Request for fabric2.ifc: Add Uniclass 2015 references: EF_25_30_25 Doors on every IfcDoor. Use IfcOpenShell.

First a look at what the model holds.

```python
import ifcopenshell

model = ifcopenshell.open("fabric2.ifc")
print(model.schema)
print("classifications:", [c.Name for c in model.by_type("IfcClassification")])
for ifc_class in ("IfcDoor", "IfcRoof", "IfcStair", "IfcWall", "IfcWindow"):
    print(ifc_class, len(model.by_type(ifc_class)))
```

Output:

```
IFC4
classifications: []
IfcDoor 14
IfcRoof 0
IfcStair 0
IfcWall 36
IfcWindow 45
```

```python
import ifcopenshell
import ifcopenshell.api.classification

model = ifcopenshell.open("fabric2.ifc")

system = ifcopenshell.api.classification.add_classification(model, classification="Uniclass 2015")

codes = {
    "IfcDoor": ("EF_25_30_25", "Doors"),
}
for ifc_class, (code, name) in codes.items():
    products = model.by_type(ifc_class)
    ifcopenshell.api.classification.add_reference(
        model, products=products, classification=system, identification=code, name=name
    )
    print(code, len(products))

model.write("fabric2_updated.ifc")
```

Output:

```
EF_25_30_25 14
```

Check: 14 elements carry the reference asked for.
